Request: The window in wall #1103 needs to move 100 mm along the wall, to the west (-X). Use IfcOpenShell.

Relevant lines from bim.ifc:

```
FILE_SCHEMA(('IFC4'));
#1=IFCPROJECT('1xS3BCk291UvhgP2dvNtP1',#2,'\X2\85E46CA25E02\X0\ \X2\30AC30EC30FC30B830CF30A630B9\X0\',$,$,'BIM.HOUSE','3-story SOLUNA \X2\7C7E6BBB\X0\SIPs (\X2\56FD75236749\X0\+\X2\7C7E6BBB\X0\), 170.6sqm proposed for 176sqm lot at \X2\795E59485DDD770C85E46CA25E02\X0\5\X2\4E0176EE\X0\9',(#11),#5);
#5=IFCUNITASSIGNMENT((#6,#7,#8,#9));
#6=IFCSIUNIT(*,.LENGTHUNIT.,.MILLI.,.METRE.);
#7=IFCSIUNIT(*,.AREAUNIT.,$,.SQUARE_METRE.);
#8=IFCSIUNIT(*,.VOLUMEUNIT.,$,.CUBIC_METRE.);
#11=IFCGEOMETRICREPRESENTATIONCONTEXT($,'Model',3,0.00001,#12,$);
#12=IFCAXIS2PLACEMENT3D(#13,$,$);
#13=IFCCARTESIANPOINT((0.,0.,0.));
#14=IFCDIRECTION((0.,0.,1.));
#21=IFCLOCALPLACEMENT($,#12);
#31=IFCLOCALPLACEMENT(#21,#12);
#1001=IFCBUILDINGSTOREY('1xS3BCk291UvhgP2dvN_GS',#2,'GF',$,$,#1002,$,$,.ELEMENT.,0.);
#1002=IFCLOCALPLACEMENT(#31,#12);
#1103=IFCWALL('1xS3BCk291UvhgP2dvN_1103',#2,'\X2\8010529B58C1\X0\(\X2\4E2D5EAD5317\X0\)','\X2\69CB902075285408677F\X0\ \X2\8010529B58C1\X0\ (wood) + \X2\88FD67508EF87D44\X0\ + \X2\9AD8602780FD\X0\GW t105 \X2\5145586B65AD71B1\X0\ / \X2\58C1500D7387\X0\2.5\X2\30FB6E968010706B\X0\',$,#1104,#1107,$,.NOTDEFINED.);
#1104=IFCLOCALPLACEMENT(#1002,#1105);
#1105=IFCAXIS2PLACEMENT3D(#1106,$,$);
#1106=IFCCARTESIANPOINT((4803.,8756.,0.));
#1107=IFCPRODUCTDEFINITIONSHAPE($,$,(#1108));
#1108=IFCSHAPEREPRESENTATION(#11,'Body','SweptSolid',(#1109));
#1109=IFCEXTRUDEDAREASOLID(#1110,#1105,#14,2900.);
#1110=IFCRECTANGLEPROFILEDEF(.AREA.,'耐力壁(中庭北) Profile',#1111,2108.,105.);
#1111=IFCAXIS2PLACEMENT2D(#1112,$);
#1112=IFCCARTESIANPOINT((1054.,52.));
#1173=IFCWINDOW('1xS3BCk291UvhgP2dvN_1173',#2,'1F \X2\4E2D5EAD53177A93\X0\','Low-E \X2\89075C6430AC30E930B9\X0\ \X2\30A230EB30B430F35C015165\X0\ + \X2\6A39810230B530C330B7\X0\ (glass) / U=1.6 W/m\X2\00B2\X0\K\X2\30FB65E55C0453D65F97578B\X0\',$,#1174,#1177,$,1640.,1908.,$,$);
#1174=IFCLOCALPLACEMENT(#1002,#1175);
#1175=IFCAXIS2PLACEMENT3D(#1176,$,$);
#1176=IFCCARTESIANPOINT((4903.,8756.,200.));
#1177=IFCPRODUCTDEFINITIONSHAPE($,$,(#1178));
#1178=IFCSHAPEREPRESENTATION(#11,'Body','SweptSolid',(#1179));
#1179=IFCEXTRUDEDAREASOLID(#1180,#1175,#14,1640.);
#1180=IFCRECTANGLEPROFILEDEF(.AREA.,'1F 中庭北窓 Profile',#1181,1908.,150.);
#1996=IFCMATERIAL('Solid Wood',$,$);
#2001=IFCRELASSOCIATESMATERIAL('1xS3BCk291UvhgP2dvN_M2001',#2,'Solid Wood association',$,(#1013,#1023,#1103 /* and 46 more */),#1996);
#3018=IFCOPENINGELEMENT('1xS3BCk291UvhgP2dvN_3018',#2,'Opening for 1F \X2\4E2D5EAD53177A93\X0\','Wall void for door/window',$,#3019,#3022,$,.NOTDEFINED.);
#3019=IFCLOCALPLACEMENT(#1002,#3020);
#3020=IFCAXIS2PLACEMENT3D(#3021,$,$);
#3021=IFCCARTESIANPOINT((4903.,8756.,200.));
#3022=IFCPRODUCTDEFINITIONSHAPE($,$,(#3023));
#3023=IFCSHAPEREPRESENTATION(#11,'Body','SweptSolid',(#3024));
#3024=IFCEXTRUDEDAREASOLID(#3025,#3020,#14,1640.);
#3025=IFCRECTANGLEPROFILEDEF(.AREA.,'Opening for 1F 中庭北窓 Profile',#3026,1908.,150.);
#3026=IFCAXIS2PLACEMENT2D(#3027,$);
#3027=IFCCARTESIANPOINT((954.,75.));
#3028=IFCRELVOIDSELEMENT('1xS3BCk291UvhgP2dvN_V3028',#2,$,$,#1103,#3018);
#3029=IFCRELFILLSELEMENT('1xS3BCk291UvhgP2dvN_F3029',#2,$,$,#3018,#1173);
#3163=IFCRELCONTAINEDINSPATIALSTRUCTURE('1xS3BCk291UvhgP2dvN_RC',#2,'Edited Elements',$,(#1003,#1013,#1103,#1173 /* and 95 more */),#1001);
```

```python
import ifcopenshell
import ifcopenshell.api.geometry
import ifcopenshell.util.placement

model = ifcopenshell.open("bim.ifc")

window = model.by_guid("1xS3BCk291UvhgP2dvN_1173")
opening = window.FillsVoids[0].RelatingOpeningElement
wall = opening.VoidsElements[0].RelatingBuildingElement

wall_matrix = ifcopenshell.util.placement.get_local_placement(wall.ObjectPlacement)
shift = wall_matrix[:3, 0] * -100.0
before = ifcopenshell.util.placement.get_local_placement(window.ObjectPlacement)[:3, 3].copy()

# The window is not placed relative to its opening, so move both.
for product in (opening, window):
    matrix = ifcopenshell.util.placement.get_local_placement(product.ObjectPlacement)
    matrix[:3, 3] += shift
    ifcopenshell.api.geometry.edit_object_placement(model, product=product, matrix=matrix, is_si=False)

after = ifcopenshell.util.placement.get_local_placement(window.ObjectPlacement)[:3, 3]
print("window moved by", (after - before).round(3) + 0.0)

model.write("bim-out.ifc")
```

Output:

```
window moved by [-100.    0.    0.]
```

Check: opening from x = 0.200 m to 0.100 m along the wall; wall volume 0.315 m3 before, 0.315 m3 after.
